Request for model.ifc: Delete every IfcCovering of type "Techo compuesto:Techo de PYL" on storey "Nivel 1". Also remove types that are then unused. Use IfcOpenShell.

First a look at what the model holds.

```python
import ifcopenshell
import ifcopenshell.util.element

model = ifcopenshell.open("model.ifc")
print(model.schema)
storey = next(s for s in model.by_type("IfcBuildingStorey") if s.Name == "Nivel 1")
coverings = [e for e in ifcopenshell.util.element.get_decomposition(storey) if e.is_a("IfcCovering")]
seen = {}
for e in coverings:
    element_type = ifcopenshell.util.element.get_type(e)
    name = element_type.Name if element_type not in (None, e) else None
    seen[name] = seen.get(name, 0) + 1
for name, count in sorted(seen.items(), key=str):
    print(count, "x", name)
```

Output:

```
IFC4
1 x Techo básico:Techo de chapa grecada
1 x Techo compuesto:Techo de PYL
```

```python
import ifcopenshell
import ifcopenshell.api.root
import ifcopenshell.util.element

model = ifcopenshell.open("model.ifc")

storey = next(s for s in model.by_type("IfcBuildingStorey") if s.Name == "Nivel 1")
coverings = [e for e in ifcopenshell.util.element.get_decomposition(storey) if e.is_a("IfcCovering")]
targets = [e for e in coverings if (t := ifcopenshell.util.element.get_type(e)) not in (None, e) and t.Name == "Techo compuesto:Techo de PYL"]
types = {ifcopenshell.util.element.get_type(e) for e in targets} - {None, *targets}

for e in targets:
    ifcopenshell.api.root.remove_product(model, product=e)
print(len(targets), "removed")

unused = [t for t in types if not ifcopenshell.util.element.get_types(t)]
for t in unused:
    ifcopenshell.api.root.remove_product(model, product=t)
print(len(unused), "unused types removed")

model.write("model_v2.ifc")
```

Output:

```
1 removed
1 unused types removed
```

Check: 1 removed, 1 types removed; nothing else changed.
